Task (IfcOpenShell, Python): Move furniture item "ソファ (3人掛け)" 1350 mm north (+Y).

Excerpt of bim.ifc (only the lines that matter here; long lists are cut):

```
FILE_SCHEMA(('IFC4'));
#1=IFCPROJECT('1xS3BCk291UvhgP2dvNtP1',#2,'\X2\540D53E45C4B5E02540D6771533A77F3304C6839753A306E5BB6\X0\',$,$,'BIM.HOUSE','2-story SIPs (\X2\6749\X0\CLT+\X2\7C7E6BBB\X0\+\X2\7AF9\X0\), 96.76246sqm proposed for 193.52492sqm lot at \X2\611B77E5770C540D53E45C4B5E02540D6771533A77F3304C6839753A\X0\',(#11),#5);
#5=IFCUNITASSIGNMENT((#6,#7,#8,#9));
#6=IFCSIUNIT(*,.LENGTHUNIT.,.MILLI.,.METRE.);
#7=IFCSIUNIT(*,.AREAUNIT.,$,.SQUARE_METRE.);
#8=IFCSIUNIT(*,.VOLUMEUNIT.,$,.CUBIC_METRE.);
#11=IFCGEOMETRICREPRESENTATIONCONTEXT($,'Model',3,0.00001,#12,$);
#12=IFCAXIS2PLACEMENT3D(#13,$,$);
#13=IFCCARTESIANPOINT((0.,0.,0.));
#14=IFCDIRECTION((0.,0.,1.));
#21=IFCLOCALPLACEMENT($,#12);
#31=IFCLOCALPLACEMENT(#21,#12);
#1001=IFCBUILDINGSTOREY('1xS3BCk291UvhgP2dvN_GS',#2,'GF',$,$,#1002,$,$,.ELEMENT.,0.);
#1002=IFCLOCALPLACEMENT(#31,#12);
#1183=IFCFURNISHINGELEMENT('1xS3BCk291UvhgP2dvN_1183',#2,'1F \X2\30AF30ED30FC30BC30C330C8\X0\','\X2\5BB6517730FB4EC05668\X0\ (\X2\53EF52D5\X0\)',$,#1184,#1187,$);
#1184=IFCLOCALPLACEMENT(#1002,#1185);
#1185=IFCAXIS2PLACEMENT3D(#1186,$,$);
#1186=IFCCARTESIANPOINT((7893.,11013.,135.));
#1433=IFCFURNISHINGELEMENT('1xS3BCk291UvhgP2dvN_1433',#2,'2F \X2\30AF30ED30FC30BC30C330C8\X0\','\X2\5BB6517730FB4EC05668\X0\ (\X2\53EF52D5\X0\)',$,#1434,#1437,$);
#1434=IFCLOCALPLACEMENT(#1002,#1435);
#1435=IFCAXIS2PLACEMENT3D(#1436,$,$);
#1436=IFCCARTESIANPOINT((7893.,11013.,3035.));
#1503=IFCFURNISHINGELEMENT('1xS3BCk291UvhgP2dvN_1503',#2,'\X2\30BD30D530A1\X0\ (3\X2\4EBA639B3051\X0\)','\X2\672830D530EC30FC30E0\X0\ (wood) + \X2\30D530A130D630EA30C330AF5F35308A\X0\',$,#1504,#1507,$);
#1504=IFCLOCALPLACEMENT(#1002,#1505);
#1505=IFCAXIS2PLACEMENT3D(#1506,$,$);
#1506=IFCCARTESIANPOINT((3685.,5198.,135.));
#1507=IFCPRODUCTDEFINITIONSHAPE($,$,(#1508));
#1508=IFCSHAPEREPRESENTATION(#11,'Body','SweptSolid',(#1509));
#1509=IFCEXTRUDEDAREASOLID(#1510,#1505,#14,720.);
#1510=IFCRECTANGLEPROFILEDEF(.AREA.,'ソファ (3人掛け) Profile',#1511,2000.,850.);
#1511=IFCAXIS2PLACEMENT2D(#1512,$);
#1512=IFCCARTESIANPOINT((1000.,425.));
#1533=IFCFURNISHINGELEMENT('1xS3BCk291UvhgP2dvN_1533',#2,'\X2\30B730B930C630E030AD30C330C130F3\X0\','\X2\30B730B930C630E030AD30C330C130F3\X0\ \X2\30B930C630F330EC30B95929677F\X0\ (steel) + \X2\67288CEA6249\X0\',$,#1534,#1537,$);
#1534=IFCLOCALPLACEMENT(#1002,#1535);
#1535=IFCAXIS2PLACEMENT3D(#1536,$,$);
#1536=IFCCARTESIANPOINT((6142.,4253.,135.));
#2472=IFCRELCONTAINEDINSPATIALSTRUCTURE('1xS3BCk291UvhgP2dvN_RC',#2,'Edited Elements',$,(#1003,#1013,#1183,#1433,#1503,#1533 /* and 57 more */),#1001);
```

```python
import ifcopenshell
import ifcopenshell.api.geometry
import ifcopenshell.util.placement
import ifcopenshell.util.unit

model = ifcopenshell.open("bim.ifc")
unit_scale = ifcopenshell.util.unit.calculate_unit_scale(model)

item = model.by_guid("1xS3BCk291UvhgP2dvN_1503")
matrix = ifcopenshell.util.placement.get_local_placement(item.ObjectPlacement)
matrix[1, 3] += 1.35 / unit_scale
ifcopenshell.api.geometry.edit_object_placement(model, product=item, matrix=matrix, is_si=False)

print(ifcopenshell.util.placement.get_local_placement(item.ObjectPlacement).round(3) + 0.0)

model.write("bim_rev.ifc")
```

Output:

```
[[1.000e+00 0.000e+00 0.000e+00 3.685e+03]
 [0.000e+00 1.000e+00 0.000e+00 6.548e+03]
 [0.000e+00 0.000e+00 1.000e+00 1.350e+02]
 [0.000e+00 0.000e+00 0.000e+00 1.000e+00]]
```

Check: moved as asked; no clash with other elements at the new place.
